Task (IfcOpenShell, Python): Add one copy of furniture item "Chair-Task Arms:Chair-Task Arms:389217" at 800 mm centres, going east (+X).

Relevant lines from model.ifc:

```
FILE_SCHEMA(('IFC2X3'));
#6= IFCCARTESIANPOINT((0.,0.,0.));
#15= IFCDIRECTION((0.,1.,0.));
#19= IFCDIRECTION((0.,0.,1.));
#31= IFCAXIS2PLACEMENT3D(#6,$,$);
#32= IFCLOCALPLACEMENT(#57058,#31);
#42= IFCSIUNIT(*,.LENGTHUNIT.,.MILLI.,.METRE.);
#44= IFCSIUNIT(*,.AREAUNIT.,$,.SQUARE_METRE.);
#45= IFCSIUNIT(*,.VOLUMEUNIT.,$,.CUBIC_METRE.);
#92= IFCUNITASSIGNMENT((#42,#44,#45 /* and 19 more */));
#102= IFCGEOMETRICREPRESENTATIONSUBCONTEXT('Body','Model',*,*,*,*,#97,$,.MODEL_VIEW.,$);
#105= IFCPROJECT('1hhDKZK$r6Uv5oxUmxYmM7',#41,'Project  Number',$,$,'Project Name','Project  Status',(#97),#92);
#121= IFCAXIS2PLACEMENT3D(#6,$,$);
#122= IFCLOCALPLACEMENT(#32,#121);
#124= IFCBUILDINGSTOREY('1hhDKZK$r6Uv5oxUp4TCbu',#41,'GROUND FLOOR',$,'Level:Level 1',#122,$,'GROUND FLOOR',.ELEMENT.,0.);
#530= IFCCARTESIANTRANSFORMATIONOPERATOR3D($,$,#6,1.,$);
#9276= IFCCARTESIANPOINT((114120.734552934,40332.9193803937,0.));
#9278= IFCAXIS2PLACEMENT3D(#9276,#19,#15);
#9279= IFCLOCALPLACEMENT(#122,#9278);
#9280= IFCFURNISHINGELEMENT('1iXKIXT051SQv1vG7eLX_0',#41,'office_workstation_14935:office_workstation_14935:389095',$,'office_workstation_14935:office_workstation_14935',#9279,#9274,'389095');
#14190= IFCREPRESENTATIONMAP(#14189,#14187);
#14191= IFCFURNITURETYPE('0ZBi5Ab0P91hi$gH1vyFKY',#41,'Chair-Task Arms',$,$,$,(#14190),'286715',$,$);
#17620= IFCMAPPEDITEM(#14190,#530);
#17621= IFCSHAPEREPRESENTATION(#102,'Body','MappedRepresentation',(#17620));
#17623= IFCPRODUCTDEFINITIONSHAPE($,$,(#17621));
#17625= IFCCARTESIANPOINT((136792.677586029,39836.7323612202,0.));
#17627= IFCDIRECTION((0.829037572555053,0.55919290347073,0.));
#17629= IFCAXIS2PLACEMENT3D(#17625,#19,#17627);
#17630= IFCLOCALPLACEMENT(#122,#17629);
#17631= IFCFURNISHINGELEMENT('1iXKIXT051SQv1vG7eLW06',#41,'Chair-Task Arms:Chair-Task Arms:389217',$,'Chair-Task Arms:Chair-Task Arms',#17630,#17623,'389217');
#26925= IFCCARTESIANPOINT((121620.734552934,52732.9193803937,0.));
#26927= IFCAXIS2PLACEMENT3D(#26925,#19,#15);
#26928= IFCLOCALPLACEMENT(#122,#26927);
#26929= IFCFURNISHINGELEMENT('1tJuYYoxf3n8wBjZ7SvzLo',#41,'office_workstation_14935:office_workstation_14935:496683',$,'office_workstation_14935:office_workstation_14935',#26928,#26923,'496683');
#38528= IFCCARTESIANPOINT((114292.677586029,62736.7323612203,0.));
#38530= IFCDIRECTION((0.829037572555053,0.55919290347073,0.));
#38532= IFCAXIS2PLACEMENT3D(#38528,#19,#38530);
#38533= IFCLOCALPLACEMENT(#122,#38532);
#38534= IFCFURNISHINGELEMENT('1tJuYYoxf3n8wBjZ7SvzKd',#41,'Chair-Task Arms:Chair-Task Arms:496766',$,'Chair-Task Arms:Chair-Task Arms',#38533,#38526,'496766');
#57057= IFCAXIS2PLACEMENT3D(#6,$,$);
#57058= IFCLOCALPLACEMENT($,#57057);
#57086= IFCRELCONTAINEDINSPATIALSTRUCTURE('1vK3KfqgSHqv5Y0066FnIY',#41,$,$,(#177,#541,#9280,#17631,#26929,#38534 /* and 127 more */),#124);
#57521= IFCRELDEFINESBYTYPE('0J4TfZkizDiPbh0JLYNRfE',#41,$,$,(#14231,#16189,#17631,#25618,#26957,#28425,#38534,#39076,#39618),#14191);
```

```python
import numpy as np
import ifcopenshell
import ifcopenshell.api.geometry
import ifcopenshell.api.root
import ifcopenshell.util.element
import ifcopenshell.util.placement

model = ifcopenshell.open("model.ifc")


def reuse_history(source, copy):
    """copy_class also copies each property set's owner history, people and application; keep the originals."""
    for rel in copy.IsDefinedBy:
        if rel.is_a("IfcRelDefinesByProperties") and (history := rel.RelatingPropertyDefinition.OwnerHistory):
            rel.RelatingPropertyDefinition.OwnerHistory = source.OwnerHistory
            ifcopenshell.util.element.remove_deep2(model, history)


source = model.by_id(17631)
base = ifcopenshell.util.placement.get_local_placement(source.ObjectPlacement)
step = np.array([1.0, 0.0, 0.0]) * 800.0

for i in range(1, 2):
    copy = ifcopenshell.api.root.copy_class(model, product=source)
    copy.Representation = ifcopenshell.util.element.copy_deep(
        model, source.Representation, exclude=["IfcGeometricRepresentationContext", "IfcRepresentationMap"]
    )
    copy.Name = "Chair-Task Arms:Chair-Task Arms"
    copy.Tag = None
    reuse_history(source, copy)
    matrix = base.copy()
    matrix[:3, 3] += i * step
    print("added at", matrix[:3, 3].round(3) + 0.0)
    ifcopenshell.api.geometry.edit_object_placement(model, product=copy, matrix=matrix, is_si=False)

model.write("model-out.ifc")
```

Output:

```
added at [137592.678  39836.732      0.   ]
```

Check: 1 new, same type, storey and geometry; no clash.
